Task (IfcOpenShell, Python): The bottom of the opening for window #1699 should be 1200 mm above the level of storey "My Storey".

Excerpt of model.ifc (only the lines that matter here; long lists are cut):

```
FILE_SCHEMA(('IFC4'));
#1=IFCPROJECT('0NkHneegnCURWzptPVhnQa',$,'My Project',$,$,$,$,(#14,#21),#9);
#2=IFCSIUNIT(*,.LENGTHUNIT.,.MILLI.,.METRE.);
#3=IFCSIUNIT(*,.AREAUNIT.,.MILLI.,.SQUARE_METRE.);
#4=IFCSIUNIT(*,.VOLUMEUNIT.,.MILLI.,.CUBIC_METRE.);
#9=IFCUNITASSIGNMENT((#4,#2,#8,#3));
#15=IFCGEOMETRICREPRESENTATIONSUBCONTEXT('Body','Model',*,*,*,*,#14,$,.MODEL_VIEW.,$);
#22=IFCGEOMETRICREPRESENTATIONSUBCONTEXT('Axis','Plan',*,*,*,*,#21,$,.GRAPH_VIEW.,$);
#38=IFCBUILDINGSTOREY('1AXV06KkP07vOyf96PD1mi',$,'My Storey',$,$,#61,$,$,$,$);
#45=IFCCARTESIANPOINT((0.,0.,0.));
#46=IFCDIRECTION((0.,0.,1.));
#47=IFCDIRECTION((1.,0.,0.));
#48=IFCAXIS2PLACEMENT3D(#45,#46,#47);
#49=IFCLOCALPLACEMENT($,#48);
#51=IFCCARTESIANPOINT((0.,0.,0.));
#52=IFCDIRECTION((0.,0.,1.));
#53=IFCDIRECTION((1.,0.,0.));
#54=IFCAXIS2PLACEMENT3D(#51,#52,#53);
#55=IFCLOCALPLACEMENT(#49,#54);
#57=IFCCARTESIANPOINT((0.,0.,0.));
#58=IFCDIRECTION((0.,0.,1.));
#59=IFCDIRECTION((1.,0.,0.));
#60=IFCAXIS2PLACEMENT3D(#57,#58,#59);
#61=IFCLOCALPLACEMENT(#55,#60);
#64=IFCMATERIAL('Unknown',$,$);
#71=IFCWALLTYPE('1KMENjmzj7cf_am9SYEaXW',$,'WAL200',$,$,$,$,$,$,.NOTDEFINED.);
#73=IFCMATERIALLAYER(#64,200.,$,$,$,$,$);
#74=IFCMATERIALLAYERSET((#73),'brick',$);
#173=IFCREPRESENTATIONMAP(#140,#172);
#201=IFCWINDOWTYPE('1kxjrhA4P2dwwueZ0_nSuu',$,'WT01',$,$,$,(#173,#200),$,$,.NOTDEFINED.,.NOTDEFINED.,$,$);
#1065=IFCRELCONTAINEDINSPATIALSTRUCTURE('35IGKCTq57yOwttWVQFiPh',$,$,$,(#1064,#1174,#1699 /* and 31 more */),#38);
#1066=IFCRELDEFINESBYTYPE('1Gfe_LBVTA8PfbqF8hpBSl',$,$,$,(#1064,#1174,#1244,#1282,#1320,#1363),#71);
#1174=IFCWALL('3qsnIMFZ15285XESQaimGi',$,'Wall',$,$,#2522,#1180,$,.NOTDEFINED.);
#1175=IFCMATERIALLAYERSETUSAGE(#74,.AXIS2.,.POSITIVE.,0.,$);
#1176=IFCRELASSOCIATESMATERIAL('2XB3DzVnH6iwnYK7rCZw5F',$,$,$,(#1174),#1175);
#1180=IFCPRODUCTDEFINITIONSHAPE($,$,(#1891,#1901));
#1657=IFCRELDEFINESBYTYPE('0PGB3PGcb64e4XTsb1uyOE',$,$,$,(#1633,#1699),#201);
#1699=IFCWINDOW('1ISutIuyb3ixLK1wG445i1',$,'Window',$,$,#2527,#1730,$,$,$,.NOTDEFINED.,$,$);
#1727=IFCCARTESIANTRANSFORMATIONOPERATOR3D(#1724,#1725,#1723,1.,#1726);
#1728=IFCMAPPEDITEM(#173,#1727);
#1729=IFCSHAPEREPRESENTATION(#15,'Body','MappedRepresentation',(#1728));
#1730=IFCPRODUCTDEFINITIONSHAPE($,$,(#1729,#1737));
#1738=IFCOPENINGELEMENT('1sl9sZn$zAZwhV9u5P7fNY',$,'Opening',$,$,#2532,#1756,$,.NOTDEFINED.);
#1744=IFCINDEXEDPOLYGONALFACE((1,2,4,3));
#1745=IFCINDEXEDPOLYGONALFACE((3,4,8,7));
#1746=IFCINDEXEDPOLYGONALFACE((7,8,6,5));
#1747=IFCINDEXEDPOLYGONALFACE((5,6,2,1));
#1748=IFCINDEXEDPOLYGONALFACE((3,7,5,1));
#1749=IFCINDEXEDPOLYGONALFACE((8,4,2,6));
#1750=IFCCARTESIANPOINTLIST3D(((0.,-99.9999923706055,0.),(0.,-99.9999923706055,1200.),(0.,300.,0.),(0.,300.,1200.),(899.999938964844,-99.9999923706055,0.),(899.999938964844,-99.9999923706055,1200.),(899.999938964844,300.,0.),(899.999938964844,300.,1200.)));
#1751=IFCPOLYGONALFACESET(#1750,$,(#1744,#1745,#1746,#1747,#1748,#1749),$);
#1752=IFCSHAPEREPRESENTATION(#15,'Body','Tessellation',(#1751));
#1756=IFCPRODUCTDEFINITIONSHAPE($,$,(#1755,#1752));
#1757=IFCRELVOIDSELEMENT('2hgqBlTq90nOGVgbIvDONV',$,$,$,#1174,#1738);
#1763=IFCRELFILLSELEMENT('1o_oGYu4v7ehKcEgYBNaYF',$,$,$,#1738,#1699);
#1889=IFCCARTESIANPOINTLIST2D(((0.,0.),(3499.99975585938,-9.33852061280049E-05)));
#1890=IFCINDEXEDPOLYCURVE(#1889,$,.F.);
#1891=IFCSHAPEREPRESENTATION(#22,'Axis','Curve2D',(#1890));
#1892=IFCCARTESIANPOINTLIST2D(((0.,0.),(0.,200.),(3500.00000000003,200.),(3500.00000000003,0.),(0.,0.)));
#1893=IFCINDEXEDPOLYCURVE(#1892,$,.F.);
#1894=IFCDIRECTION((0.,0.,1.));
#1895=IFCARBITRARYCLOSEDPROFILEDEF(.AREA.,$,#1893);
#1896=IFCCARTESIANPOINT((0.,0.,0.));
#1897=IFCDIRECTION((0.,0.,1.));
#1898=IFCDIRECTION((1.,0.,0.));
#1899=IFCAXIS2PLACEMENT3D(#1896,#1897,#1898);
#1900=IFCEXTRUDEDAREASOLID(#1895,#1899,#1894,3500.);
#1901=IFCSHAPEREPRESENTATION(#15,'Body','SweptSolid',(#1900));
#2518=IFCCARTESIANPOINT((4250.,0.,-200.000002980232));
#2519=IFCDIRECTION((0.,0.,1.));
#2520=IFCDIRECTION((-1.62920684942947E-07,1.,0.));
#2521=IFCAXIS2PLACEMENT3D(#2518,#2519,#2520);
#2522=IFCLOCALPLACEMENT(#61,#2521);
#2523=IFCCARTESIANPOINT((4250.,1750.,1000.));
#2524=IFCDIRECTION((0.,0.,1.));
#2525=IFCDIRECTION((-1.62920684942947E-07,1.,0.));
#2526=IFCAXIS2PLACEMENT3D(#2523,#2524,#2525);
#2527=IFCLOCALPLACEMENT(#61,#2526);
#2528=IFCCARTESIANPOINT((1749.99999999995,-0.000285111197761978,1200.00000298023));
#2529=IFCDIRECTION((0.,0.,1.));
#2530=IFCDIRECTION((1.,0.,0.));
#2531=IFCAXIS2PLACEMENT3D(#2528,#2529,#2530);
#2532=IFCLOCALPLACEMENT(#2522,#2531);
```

```python
import numpy as np
import ifcopenshell
import ifcopenshell.api.geometry
import ifcopenshell.geom
import ifcopenshell.util.element
import ifcopenshell.util.placement
import ifcopenshell.util.shape
import ifcopenshell.util.unit

model = ifcopenshell.open("model.ifc")
unit_scale = ifcopenshell.util.unit.calculate_unit_scale(model)

window = model.by_id(1699)
opening = window.FillsVoids[0].RelatingOpeningElement
storey = ifcopenshell.util.element.get_container(window, ifc_class="IfcBuildingStorey")
level = ifcopenshell.util.placement.get_local_placement(storey.ObjectPlacement)[2, 3]

# The opening's origin need not be at the sill, so measure its lowest point.
shape = ifcopenshell.geom.create_shape(ifcopenshell.geom.settings(), opening)
bottom = ifcopenshell.util.shape.get_shape_bottom_elevation(shape, shape.geometry) / unit_scale
dz = level + 1.2 / unit_scale - bottom

shift = np.array([0.0, 0.0, dz])
# The window is not placed relative to its opening, so move both.
for product in (opening, window):
    matrix = ifcopenshell.util.placement.get_local_placement(product.ObjectPlacement)
    matrix[:3, 3] += shift
    ifcopenshell.api.geometry.edit_object_placement(model, product=product, matrix=matrix, is_si=False)

print(f"moved by {dz * unit_scale:+.3f} m")

model.write("model_rev.ifc")
```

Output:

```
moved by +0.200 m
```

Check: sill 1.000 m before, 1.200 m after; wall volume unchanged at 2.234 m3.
